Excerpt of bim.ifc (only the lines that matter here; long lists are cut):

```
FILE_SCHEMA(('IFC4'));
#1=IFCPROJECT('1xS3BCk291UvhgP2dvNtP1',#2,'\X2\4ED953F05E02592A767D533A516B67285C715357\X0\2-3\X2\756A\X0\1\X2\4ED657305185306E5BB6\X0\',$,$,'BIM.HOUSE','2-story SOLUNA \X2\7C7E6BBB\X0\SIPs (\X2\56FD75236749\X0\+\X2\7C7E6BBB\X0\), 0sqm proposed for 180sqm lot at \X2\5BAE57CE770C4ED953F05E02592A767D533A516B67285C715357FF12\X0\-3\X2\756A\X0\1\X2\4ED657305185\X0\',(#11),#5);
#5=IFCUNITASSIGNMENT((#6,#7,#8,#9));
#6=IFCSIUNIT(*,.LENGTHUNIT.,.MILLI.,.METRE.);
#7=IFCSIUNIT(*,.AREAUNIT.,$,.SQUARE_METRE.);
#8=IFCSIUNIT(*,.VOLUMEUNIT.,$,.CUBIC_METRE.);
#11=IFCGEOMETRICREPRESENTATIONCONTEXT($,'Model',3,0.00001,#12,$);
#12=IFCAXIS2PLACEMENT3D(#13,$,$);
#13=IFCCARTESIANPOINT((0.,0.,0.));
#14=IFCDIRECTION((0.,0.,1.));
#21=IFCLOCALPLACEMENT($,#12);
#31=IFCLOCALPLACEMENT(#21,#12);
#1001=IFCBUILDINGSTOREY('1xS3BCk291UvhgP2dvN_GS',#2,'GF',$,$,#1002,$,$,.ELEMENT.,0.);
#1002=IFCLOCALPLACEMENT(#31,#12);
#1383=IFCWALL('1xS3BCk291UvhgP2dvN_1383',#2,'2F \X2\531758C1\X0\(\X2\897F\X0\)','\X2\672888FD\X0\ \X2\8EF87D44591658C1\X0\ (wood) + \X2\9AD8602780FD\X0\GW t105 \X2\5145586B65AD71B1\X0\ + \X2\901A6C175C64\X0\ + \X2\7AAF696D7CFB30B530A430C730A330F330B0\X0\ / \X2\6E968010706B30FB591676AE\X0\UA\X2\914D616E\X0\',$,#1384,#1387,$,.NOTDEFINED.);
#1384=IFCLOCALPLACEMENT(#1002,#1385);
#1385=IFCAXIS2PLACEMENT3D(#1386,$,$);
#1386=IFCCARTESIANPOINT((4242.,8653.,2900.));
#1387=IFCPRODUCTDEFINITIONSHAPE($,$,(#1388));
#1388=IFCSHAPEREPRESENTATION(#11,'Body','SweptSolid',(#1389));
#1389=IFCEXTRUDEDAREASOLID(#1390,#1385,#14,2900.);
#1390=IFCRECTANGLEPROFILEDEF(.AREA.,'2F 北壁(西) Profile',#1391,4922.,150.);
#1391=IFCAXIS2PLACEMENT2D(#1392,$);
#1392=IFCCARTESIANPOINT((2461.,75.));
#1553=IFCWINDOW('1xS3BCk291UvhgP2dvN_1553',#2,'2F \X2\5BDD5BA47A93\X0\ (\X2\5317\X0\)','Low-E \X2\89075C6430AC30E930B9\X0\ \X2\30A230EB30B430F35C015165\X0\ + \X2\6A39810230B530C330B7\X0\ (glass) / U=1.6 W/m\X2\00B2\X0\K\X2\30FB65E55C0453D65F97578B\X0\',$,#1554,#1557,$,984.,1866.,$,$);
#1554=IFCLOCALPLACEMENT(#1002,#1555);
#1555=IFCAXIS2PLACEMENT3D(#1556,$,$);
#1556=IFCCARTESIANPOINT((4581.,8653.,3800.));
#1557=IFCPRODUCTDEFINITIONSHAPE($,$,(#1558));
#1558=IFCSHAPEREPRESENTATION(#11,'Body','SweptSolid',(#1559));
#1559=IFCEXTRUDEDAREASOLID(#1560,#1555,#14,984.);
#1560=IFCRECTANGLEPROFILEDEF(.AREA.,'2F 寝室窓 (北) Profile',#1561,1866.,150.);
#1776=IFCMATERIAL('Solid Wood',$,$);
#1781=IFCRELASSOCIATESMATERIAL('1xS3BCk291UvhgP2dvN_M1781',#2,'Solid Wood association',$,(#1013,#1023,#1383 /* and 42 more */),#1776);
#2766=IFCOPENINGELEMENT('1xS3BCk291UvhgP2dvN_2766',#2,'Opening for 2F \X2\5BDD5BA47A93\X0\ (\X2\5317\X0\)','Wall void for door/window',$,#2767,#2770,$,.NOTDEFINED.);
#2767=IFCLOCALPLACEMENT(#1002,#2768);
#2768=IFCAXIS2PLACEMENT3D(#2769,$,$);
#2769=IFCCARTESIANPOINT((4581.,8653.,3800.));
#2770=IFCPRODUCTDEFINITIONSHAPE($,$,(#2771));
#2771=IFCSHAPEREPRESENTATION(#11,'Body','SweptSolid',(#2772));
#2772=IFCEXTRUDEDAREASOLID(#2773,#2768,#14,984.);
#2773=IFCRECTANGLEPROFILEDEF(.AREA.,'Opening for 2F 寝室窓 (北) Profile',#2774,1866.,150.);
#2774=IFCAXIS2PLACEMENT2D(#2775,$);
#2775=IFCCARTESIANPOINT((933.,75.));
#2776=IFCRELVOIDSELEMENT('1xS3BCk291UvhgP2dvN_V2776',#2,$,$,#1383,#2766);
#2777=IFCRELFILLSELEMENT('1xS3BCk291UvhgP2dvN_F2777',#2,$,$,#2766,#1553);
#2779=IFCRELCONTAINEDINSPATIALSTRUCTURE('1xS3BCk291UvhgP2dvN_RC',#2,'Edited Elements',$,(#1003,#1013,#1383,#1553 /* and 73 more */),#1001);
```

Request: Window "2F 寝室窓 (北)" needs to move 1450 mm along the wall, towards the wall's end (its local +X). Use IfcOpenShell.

```python
import ifcopenshell
import ifcopenshell.api.geometry
import ifcopenshell.util.placement

model = ifcopenshell.open("bim.ifc")

window = model.by_guid("1xS3BCk291UvhgP2dvN_1553")
opening = window.FillsVoids[0].RelatingOpeningElement
wall = opening.VoidsElements[0].RelatingBuildingElement

wall_matrix = ifcopenshell.util.placement.get_local_placement(wall.ObjectPlacement)
shift = wall_matrix[:3, 0] * 1450.0
before = ifcopenshell.util.placement.get_local_placement(window.ObjectPlacement)[:3, 3].copy()

# The window is not placed relative to its opening, so move both.
for product in (opening, window):
    matrix = ifcopenshell.util.placement.get_local_placement(product.ObjectPlacement)
    matrix[:3, 3] += shift
    ifcopenshell.api.geometry.edit_object_placement(model, product=product, matrix=matrix, is_si=False)

after = ifcopenshell.util.placement.get_local_placement(window.ObjectPlacement)[:3, 3]
print("window moved by", (after - before).round(3) + 0.0)

model.write("bim_rev.ifc")
```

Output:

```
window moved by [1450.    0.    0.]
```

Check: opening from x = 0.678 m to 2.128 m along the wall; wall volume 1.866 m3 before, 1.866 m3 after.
